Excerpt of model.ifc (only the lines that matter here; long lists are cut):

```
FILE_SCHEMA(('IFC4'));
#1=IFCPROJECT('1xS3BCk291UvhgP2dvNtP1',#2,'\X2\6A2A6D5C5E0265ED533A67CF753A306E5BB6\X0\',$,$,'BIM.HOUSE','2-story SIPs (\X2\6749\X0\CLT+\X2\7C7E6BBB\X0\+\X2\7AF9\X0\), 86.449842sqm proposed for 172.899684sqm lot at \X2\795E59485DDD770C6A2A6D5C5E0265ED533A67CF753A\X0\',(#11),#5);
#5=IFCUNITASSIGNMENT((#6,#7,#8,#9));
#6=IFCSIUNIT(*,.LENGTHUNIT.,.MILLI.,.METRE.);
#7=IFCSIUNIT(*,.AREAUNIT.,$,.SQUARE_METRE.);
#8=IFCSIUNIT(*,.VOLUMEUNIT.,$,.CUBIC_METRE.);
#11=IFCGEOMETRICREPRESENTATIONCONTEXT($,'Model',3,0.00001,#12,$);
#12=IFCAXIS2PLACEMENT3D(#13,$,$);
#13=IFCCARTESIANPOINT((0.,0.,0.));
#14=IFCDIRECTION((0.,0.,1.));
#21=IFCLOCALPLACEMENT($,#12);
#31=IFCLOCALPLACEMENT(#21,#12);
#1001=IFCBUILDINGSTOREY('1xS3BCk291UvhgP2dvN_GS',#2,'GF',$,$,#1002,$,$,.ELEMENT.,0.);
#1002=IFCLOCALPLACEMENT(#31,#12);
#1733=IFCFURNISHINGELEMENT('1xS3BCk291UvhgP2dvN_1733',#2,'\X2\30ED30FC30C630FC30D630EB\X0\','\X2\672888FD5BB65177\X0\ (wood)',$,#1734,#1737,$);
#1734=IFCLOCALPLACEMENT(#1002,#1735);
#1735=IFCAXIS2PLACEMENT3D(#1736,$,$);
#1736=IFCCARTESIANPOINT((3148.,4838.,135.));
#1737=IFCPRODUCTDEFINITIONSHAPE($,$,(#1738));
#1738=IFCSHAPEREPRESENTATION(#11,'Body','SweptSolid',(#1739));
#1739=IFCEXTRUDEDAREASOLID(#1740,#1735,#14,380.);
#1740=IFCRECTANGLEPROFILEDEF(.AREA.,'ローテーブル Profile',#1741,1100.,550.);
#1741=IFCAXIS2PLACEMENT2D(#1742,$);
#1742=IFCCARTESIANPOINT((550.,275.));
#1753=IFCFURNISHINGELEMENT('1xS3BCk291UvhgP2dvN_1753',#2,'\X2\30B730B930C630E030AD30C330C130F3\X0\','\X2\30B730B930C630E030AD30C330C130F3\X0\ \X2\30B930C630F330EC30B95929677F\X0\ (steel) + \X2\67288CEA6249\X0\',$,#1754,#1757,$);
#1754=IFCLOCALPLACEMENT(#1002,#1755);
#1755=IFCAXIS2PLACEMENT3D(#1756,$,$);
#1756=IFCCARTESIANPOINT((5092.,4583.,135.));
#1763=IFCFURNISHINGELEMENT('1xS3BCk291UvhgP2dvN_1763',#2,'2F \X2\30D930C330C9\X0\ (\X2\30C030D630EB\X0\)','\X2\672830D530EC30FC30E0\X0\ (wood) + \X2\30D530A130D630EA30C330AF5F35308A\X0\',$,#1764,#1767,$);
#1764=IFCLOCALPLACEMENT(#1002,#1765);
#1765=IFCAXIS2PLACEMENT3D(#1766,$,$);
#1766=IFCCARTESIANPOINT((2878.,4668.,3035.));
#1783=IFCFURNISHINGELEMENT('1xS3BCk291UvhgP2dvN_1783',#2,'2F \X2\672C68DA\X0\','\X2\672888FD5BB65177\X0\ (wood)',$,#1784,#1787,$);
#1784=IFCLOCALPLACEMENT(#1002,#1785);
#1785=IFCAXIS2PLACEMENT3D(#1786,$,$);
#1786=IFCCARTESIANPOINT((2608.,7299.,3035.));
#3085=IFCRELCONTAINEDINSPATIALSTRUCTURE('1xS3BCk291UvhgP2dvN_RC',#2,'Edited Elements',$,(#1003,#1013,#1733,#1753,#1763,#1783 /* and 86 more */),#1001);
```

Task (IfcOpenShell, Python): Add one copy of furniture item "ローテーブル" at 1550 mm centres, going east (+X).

```python
import numpy as np
import ifcopenshell
import ifcopenshell.api.geometry
import ifcopenshell.api.root
import ifcopenshell.util.element
import ifcopenshell.util.placement
import ifcopenshell.util.unit

model = ifcopenshell.open("model.ifc")
unit_scale = ifcopenshell.util.unit.calculate_unit_scale(model)


def reuse_history(source, copy):
    """copy_class also copies each property set's owner history, people and application; keep the originals."""
    for rel in copy.IsDefinedBy:
        if rel.is_a("IfcRelDefinesByProperties") and (history := rel.RelatingPropertyDefinition.OwnerHistory):
            rel.RelatingPropertyDefinition.OwnerHistory = source.OwnerHistory
            ifcopenshell.util.element.remove_deep2(model, history)


source = model.by_guid("1xS3BCk291UvhgP2dvN_1733")
base = ifcopenshell.util.placement.get_local_placement(source.ObjectPlacement)
step = np.array([1.0, 0.0, 0.0]) * 1.55 / unit_scale

for i in range(1, 2):
    copy = ifcopenshell.api.root.copy_class(model, product=source)
    copy.Representation = ifcopenshell.util.element.copy_deep(
        model, source.Representation, exclude=["IfcGeometricRepresentationContext", "IfcRepresentationMap"]
    )
    reuse_history(source, copy)
    matrix = base.copy()
    matrix[:3, 3] += i * step
    print("added at", matrix[:3, 3].round(3) + 0.0)
    ifcopenshell.api.geometry.edit_object_placement(model, product=copy, matrix=matrix, is_si=False)

model.write("model_rev.ifc")
```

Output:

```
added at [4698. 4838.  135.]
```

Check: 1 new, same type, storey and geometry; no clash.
